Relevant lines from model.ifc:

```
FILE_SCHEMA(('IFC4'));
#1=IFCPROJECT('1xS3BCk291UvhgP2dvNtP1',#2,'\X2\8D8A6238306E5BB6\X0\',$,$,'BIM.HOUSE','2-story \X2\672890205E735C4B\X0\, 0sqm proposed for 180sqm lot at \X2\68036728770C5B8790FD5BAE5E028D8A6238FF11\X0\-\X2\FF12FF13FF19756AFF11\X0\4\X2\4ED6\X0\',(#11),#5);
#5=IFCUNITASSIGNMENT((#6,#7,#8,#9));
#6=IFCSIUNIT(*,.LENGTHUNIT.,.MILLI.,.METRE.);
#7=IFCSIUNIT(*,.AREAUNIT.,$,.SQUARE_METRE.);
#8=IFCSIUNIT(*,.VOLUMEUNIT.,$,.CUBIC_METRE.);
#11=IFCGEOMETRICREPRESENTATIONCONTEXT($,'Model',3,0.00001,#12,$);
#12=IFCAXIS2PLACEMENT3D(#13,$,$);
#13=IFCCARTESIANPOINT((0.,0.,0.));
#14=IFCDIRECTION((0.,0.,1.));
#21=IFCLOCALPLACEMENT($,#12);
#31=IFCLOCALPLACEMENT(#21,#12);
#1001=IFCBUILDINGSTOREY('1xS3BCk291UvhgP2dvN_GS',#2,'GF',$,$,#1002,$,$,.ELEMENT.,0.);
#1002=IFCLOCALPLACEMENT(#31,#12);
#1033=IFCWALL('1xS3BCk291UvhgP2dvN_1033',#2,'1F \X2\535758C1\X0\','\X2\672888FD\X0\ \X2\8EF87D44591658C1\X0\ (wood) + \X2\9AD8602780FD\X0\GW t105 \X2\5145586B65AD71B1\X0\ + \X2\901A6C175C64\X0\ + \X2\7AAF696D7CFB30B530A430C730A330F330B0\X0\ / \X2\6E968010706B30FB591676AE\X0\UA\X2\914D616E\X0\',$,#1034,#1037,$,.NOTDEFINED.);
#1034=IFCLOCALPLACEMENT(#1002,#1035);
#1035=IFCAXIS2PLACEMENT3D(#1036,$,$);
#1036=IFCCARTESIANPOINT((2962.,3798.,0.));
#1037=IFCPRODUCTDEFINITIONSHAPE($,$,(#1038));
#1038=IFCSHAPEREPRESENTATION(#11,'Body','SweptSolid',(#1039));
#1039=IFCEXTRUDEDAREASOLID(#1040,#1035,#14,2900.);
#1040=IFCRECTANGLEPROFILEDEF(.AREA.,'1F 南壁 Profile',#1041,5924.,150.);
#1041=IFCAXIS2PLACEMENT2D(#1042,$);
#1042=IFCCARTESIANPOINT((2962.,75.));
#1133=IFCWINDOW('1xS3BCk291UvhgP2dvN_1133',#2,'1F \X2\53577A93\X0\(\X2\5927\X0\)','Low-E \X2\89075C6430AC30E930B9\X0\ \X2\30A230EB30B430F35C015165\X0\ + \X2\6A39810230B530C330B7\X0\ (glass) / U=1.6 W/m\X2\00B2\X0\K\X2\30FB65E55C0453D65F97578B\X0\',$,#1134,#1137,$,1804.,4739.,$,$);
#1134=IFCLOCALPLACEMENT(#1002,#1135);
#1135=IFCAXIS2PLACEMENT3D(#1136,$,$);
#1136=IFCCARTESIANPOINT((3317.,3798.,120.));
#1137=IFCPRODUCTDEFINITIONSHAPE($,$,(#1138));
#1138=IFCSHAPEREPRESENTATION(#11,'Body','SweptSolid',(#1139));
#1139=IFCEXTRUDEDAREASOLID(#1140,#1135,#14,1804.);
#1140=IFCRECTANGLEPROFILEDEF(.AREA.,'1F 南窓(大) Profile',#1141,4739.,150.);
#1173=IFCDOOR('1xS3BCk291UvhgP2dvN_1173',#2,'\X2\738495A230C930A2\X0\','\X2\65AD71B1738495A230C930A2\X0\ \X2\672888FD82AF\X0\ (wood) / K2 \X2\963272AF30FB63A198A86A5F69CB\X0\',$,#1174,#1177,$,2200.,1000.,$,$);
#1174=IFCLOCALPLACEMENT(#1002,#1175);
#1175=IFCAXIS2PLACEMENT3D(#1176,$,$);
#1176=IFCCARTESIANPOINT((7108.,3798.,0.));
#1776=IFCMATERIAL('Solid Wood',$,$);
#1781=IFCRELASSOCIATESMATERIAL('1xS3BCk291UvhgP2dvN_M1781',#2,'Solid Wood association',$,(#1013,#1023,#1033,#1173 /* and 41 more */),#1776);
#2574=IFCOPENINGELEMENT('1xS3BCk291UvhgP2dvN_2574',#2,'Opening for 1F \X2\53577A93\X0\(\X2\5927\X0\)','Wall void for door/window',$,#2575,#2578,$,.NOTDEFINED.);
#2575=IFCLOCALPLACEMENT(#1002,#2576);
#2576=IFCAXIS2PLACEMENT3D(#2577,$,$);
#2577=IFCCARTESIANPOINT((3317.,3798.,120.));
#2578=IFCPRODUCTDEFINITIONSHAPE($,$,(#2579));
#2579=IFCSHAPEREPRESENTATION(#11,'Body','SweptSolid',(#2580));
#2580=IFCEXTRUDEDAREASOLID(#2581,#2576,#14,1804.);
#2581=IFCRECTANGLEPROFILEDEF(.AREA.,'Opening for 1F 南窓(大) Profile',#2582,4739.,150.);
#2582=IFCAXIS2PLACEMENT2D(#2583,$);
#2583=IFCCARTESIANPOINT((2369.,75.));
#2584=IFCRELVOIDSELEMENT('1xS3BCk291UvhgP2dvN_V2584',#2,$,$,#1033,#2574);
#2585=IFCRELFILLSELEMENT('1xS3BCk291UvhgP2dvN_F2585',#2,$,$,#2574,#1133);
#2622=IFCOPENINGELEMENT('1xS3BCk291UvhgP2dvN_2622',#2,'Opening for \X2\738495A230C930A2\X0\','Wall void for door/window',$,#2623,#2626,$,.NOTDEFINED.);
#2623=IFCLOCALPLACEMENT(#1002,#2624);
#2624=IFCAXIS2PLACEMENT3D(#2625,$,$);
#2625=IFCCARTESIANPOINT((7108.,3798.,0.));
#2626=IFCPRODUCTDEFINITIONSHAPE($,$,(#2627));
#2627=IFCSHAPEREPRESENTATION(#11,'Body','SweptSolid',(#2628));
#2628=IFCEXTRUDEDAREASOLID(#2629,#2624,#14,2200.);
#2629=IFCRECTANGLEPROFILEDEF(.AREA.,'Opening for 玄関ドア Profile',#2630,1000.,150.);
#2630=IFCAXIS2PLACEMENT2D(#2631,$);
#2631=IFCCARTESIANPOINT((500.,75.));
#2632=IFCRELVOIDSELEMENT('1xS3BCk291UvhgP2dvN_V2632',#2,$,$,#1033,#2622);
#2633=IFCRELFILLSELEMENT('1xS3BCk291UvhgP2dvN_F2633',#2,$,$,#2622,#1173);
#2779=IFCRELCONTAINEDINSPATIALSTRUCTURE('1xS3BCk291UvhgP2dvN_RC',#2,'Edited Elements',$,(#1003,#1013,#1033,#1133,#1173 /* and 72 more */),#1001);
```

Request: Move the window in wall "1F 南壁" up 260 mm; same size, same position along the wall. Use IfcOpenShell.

```python
import numpy as np
import ifcopenshell
import ifcopenshell.api.geometry
import ifcopenshell.util.placement
import ifcopenshell.util.unit

model = ifcopenshell.open("model.ifc")
unit_scale = ifcopenshell.util.unit.calculate_unit_scale(model)

window = model.by_guid("1xS3BCk291UvhgP2dvN_1133")
opening = window.FillsVoids[0].RelatingOpeningElement
dz = 0.26 / unit_scale

shift = np.array([0.0, 0.0, dz])
# The window is not placed relative to its opening, so move both.
for product in (opening, window):
    matrix = ifcopenshell.util.placement.get_local_placement(product.ObjectPlacement)
    matrix[:3, 3] += shift
    ifcopenshell.api.geometry.edit_object_placement(model, product=product, matrix=matrix, is_si=False)

print(f"moved by {dz * unit_scale:+.3f} m")

model.write("model_updated.ifc")
```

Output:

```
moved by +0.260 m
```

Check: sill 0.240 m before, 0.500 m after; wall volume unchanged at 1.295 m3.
